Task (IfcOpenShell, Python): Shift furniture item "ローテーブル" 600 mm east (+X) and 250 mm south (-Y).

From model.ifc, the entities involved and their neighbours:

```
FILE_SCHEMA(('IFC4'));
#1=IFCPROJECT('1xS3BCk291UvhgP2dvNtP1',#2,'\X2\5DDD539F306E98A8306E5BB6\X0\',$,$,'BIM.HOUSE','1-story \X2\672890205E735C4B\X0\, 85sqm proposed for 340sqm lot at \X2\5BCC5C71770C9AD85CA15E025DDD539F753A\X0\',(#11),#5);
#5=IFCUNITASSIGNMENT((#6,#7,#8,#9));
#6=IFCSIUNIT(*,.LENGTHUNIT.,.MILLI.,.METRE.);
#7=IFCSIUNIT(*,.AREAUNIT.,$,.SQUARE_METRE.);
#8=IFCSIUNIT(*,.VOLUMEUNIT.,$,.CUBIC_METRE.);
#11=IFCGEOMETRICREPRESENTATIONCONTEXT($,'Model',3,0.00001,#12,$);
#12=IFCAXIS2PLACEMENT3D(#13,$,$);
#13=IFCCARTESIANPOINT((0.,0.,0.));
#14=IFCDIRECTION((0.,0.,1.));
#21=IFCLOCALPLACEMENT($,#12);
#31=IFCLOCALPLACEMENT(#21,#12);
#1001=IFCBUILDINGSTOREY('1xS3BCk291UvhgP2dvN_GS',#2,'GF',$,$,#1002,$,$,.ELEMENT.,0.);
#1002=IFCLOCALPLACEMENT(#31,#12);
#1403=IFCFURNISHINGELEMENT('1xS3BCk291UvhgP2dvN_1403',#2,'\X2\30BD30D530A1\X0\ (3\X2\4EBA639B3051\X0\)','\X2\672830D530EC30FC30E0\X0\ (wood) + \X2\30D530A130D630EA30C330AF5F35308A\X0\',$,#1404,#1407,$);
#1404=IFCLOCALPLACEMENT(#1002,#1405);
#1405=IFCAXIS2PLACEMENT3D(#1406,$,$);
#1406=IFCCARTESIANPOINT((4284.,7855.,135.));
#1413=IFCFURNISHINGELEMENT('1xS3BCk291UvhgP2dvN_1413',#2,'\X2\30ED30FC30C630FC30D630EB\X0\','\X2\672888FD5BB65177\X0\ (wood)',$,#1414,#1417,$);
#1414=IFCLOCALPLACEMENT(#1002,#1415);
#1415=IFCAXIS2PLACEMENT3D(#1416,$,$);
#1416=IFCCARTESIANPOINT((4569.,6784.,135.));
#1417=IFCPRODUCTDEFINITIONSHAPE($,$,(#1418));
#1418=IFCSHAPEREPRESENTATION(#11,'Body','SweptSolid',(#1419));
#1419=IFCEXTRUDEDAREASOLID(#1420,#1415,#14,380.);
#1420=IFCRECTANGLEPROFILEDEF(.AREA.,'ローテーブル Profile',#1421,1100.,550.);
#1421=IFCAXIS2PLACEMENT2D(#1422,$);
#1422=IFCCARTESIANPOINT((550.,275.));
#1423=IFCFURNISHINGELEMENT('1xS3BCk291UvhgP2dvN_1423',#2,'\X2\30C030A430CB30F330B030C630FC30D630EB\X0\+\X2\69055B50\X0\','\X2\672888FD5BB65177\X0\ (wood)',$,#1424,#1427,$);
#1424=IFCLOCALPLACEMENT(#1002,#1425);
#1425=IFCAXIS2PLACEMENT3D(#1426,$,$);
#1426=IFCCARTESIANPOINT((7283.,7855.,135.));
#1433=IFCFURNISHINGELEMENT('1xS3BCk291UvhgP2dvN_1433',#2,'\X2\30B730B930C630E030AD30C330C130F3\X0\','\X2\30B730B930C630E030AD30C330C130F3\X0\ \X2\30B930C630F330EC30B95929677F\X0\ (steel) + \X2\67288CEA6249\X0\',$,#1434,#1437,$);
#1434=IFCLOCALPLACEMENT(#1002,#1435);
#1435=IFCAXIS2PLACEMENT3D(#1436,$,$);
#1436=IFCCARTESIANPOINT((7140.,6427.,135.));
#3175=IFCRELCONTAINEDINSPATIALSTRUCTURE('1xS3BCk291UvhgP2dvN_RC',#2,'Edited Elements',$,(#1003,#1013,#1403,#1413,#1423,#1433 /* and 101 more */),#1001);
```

```python
import ifcopenshell
import ifcopenshell.api.geometry
import ifcopenshell.util.placement

model = ifcopenshell.open("model.ifc")

item = model.by_guid("1xS3BCk291UvhgP2dvN_1413")
matrix = ifcopenshell.util.placement.get_local_placement(item.ObjectPlacement)
matrix[0, 3] += 600.0
matrix[1, 3] -= 250.0
ifcopenshell.api.geometry.edit_object_placement(model, product=item, matrix=matrix, is_si=False)

print(ifcopenshell.util.placement.get_local_placement(item.ObjectPlacement).round(3) + 0.0)

model.write("model_edited.ifc")
```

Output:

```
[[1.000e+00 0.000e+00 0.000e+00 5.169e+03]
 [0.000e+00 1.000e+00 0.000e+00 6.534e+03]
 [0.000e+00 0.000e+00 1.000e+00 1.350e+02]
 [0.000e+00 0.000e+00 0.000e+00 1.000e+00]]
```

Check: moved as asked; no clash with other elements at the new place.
